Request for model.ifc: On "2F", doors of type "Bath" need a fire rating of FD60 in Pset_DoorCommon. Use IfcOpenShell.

First a look at what the model holds.

```python
import ifcopenshell
import ifcopenshell.util.element

model = ifcopenshell.open("model.ifc")
print(model.schema)
storey = next(s for s in model.by_type("IfcBuildingStorey") if s.Name == "2F")
doors = [e for e in ifcopenshell.util.element.get_decomposition(storey) if e.is_a("IfcDoor")]
seen = {}
for e in doors:
    element_type = ifcopenshell.util.element.get_type(e)
    key = (element_type.Name if element_type != e and element_type else None, ifcopenshell.util.element.get_pset(e, "Pset_DoorCommon", "FireRating"))
    seen[key] = seen.get(key, 0) + 1
for (name, value), count in sorted(seen.items(), key=str):
    print(count, "x", name, "|", value)
```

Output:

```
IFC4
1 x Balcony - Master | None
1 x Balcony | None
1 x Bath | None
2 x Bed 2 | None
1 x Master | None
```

```python
import ifcopenshell
import ifcopenshell.api.pset
import ifcopenshell.util.element

model = ifcopenshell.open("model.ifc")

storey = next(s for s in model.by_type("IfcBuildingStorey") if s.Name == "2F")
doors = [e for e in ifcopenshell.util.element.get_decomposition(storey) if e.is_a("IfcDoor")]

count = 0
for e in doors:
    element_type = ifcopenshell.util.element.get_type(e)
    if element_type in (None, e) or element_type.Name != "Bath":
        continue
    # add_pset returns the element's existing set when there is one.
    pset = ifcopenshell.api.pset.add_pset(model, product=e, name="Pset_DoorCommon")
    ifcopenshell.api.pset.edit_pset(model, pset=pset, properties={"FireRating": "FD60"})
    count += 1

print(count, "doors updated")

model.write("model-out.ifc")
```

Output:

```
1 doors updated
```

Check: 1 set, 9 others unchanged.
